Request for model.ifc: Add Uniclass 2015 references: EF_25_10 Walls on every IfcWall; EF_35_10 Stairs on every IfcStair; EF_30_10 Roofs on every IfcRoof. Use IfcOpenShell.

First a look at what the model holds.

```python
import ifcopenshell

model = ifcopenshell.open("model.ifc")
print(model.schema)
print("classifications:", [c.Name for c in model.by_type("IfcClassification")])
for ifc_class in ("IfcDoor", "IfcRoof", "IfcStair", "IfcWall", "IfcWindow"):
    print(ifc_class, len(model.by_type(ifc_class)))
```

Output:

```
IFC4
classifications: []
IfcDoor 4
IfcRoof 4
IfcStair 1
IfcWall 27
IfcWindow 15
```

```python
import ifcopenshell
import ifcopenshell.api.classification

model = ifcopenshell.open("model.ifc")

system = ifcopenshell.api.classification.add_classification(model, classification="Uniclass 2015")

codes = {
    "IfcWall": ("EF_25_10", "Walls"),
    "IfcStair": ("EF_35_10", "Stairs"),
    "IfcRoof": ("EF_30_10", "Roofs"),
}
for ifc_class, (code, name) in codes.items():
    products = model.by_type(ifc_class)
    ifcopenshell.api.classification.add_reference(
        model, products=products, classification=system, identification=code, name=name
    )
    print(code, len(products))

model.write("model_v2.ifc")
```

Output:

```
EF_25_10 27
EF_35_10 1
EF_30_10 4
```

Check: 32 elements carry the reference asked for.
